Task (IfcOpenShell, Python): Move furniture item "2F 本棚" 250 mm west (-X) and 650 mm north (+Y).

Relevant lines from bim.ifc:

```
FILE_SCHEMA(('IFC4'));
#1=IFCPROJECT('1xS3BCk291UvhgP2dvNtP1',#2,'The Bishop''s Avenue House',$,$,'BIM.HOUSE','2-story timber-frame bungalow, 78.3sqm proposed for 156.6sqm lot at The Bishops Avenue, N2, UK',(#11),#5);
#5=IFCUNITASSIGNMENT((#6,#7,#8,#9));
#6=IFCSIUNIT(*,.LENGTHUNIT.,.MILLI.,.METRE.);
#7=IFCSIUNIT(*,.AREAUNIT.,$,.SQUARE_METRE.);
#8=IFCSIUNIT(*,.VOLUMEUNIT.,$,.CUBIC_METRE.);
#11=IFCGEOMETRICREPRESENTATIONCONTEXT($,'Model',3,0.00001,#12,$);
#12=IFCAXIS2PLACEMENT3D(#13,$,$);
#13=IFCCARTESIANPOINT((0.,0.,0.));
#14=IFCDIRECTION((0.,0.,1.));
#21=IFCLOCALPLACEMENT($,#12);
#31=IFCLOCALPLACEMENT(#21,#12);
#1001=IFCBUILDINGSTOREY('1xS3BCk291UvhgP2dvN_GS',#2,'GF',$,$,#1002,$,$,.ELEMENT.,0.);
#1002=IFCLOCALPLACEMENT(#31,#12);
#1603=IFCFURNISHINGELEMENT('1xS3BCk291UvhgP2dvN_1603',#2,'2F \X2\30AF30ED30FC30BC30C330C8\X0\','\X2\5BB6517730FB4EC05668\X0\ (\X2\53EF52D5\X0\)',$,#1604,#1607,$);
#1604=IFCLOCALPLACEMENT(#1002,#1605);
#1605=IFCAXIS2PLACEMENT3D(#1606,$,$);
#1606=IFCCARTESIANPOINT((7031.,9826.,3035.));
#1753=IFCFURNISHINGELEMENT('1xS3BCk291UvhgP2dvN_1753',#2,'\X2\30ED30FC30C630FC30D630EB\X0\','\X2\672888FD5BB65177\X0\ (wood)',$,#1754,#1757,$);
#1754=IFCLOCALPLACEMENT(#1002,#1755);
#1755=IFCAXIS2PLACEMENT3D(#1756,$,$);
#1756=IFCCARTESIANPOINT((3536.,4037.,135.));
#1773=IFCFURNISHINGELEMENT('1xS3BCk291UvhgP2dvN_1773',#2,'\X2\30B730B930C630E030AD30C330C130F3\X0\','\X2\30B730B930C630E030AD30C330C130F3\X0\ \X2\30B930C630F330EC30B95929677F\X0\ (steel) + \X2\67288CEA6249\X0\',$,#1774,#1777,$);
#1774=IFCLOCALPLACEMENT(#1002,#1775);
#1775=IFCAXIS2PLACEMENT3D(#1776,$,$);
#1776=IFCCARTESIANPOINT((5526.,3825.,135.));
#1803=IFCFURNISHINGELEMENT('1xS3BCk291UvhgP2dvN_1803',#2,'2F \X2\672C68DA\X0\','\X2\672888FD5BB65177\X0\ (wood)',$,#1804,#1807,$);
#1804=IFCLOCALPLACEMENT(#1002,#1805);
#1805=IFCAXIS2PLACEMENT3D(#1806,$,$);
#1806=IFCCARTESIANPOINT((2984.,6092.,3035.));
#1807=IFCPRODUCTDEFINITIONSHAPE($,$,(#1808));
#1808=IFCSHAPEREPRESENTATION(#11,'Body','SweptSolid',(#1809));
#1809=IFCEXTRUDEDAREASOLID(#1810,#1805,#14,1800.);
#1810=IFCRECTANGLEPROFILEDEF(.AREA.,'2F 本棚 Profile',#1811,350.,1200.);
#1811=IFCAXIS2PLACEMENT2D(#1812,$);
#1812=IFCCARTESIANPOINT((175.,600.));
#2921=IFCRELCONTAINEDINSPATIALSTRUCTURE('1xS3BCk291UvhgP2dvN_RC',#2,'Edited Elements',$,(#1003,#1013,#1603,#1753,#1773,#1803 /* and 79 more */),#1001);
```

```python
import ifcopenshell
import ifcopenshell.api.geometry
import ifcopenshell.util.placement
import ifcopenshell.util.unit

model = ifcopenshell.open("bim.ifc")
unit_scale = ifcopenshell.util.unit.calculate_unit_scale(model)

item = model.by_guid("1xS3BCk291UvhgP2dvN_1803")
matrix = ifcopenshell.util.placement.get_local_placement(item.ObjectPlacement)
matrix[0, 3] -= 0.25 / unit_scale
matrix[1, 3] += 0.65 / unit_scale
ifcopenshell.api.geometry.edit_object_placement(model, product=item, matrix=matrix, is_si=False)

print(ifcopenshell.util.placement.get_local_placement(item.ObjectPlacement).round(3) + 0.0)

model.write("bim_edited.ifc")
```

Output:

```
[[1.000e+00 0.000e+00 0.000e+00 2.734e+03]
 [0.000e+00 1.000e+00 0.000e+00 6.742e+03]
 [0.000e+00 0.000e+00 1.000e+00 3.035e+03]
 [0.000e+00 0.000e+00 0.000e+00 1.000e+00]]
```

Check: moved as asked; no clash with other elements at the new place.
